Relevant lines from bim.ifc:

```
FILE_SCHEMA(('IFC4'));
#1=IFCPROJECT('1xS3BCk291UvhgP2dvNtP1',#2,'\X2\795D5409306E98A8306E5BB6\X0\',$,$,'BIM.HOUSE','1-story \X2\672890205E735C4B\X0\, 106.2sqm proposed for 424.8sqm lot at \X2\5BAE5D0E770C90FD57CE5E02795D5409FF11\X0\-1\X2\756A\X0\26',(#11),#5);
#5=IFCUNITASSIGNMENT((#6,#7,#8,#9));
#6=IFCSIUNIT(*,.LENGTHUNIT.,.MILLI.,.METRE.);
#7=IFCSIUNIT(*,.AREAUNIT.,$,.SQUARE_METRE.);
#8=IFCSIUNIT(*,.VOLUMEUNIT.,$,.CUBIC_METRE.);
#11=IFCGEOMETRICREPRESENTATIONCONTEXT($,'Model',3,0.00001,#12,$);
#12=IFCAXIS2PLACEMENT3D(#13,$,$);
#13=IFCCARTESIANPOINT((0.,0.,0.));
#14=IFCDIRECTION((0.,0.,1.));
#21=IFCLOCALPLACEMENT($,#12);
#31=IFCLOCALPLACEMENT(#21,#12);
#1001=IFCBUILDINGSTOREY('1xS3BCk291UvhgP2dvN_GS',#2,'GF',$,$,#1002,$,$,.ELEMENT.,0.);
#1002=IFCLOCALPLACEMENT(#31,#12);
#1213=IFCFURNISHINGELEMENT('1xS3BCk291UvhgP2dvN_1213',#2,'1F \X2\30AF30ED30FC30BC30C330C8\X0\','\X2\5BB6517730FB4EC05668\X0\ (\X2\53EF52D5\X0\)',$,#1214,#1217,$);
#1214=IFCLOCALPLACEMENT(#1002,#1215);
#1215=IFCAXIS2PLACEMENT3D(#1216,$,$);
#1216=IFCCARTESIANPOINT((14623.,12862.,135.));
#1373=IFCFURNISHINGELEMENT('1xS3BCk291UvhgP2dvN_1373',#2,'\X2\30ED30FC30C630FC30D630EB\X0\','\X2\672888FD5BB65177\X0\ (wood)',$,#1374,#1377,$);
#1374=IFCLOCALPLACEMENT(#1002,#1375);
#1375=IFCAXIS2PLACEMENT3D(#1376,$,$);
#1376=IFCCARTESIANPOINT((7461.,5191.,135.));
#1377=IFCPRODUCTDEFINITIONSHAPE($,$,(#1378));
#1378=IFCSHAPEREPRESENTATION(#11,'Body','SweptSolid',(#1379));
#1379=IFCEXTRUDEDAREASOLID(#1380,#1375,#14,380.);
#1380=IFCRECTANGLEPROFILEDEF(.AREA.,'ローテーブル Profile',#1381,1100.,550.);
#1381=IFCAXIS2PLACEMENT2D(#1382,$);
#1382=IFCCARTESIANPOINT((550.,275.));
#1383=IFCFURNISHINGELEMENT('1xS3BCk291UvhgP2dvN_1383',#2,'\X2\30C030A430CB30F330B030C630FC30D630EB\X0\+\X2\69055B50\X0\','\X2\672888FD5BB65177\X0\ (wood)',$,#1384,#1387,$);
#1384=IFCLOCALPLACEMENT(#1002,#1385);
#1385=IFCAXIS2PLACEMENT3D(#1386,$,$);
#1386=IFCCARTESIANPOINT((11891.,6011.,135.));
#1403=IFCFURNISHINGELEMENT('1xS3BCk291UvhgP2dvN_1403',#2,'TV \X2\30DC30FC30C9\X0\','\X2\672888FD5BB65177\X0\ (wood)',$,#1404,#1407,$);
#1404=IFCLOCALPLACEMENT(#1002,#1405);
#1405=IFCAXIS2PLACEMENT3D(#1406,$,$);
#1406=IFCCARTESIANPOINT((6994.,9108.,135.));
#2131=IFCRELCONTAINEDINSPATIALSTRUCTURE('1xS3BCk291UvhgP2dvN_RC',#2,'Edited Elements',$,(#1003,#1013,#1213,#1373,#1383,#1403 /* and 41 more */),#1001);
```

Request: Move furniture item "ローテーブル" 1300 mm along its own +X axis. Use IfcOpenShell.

```python
import ifcopenshell
import ifcopenshell.api.geometry
import ifcopenshell.util.placement

model = ifcopenshell.open("bim.ifc")

item = model.by_id(1373)
matrix = ifcopenshell.util.placement.get_local_placement(item.ObjectPlacement)
matrix[:3, 3] += matrix[:3, 0] * 1300.0
ifcopenshell.api.geometry.edit_object_placement(model, product=item, matrix=matrix, is_si=False)

print(ifcopenshell.util.placement.get_local_placement(item.ObjectPlacement).round(3) + 0.0)

model.write("bim-out.ifc")
```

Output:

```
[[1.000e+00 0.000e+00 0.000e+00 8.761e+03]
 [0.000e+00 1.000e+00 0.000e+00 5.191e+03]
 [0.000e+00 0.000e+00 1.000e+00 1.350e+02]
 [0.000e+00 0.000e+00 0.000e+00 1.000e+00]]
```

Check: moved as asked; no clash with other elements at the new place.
